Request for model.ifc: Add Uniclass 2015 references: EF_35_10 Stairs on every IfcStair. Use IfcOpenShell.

First a look at what the model holds.

```python
import ifcopenshell

model = ifcopenshell.open("model.ifc")
print(model.schema)
print("classifications:", [c.Name for c in model.by_type("IfcClassification")])
for ifc_class in ("IfcDoor", "IfcRoof", "IfcStair", "IfcWall", "IfcWindow"):
    print(ifc_class, len(model.by_type(ifc_class)))
```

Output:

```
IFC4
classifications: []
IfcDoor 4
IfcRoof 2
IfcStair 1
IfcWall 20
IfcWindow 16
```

```python
import ifcopenshell
import ifcopenshell.api.classification

model = ifcopenshell.open("model.ifc")

system = ifcopenshell.api.classification.add_classification(model, classification="Uniclass 2015")

codes = {
    "IfcStair": ("EF_35_10", "Stairs"),
}
for ifc_class, (code, name) in codes.items():
    products = model.by_type(ifc_class)
    ifcopenshell.api.classification.add_reference(
        model, products=products, classification=system, identification=code, name=name
    )
    print(code, len(products))

model.write("model_edited.ifc")
```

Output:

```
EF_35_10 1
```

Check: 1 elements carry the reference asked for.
